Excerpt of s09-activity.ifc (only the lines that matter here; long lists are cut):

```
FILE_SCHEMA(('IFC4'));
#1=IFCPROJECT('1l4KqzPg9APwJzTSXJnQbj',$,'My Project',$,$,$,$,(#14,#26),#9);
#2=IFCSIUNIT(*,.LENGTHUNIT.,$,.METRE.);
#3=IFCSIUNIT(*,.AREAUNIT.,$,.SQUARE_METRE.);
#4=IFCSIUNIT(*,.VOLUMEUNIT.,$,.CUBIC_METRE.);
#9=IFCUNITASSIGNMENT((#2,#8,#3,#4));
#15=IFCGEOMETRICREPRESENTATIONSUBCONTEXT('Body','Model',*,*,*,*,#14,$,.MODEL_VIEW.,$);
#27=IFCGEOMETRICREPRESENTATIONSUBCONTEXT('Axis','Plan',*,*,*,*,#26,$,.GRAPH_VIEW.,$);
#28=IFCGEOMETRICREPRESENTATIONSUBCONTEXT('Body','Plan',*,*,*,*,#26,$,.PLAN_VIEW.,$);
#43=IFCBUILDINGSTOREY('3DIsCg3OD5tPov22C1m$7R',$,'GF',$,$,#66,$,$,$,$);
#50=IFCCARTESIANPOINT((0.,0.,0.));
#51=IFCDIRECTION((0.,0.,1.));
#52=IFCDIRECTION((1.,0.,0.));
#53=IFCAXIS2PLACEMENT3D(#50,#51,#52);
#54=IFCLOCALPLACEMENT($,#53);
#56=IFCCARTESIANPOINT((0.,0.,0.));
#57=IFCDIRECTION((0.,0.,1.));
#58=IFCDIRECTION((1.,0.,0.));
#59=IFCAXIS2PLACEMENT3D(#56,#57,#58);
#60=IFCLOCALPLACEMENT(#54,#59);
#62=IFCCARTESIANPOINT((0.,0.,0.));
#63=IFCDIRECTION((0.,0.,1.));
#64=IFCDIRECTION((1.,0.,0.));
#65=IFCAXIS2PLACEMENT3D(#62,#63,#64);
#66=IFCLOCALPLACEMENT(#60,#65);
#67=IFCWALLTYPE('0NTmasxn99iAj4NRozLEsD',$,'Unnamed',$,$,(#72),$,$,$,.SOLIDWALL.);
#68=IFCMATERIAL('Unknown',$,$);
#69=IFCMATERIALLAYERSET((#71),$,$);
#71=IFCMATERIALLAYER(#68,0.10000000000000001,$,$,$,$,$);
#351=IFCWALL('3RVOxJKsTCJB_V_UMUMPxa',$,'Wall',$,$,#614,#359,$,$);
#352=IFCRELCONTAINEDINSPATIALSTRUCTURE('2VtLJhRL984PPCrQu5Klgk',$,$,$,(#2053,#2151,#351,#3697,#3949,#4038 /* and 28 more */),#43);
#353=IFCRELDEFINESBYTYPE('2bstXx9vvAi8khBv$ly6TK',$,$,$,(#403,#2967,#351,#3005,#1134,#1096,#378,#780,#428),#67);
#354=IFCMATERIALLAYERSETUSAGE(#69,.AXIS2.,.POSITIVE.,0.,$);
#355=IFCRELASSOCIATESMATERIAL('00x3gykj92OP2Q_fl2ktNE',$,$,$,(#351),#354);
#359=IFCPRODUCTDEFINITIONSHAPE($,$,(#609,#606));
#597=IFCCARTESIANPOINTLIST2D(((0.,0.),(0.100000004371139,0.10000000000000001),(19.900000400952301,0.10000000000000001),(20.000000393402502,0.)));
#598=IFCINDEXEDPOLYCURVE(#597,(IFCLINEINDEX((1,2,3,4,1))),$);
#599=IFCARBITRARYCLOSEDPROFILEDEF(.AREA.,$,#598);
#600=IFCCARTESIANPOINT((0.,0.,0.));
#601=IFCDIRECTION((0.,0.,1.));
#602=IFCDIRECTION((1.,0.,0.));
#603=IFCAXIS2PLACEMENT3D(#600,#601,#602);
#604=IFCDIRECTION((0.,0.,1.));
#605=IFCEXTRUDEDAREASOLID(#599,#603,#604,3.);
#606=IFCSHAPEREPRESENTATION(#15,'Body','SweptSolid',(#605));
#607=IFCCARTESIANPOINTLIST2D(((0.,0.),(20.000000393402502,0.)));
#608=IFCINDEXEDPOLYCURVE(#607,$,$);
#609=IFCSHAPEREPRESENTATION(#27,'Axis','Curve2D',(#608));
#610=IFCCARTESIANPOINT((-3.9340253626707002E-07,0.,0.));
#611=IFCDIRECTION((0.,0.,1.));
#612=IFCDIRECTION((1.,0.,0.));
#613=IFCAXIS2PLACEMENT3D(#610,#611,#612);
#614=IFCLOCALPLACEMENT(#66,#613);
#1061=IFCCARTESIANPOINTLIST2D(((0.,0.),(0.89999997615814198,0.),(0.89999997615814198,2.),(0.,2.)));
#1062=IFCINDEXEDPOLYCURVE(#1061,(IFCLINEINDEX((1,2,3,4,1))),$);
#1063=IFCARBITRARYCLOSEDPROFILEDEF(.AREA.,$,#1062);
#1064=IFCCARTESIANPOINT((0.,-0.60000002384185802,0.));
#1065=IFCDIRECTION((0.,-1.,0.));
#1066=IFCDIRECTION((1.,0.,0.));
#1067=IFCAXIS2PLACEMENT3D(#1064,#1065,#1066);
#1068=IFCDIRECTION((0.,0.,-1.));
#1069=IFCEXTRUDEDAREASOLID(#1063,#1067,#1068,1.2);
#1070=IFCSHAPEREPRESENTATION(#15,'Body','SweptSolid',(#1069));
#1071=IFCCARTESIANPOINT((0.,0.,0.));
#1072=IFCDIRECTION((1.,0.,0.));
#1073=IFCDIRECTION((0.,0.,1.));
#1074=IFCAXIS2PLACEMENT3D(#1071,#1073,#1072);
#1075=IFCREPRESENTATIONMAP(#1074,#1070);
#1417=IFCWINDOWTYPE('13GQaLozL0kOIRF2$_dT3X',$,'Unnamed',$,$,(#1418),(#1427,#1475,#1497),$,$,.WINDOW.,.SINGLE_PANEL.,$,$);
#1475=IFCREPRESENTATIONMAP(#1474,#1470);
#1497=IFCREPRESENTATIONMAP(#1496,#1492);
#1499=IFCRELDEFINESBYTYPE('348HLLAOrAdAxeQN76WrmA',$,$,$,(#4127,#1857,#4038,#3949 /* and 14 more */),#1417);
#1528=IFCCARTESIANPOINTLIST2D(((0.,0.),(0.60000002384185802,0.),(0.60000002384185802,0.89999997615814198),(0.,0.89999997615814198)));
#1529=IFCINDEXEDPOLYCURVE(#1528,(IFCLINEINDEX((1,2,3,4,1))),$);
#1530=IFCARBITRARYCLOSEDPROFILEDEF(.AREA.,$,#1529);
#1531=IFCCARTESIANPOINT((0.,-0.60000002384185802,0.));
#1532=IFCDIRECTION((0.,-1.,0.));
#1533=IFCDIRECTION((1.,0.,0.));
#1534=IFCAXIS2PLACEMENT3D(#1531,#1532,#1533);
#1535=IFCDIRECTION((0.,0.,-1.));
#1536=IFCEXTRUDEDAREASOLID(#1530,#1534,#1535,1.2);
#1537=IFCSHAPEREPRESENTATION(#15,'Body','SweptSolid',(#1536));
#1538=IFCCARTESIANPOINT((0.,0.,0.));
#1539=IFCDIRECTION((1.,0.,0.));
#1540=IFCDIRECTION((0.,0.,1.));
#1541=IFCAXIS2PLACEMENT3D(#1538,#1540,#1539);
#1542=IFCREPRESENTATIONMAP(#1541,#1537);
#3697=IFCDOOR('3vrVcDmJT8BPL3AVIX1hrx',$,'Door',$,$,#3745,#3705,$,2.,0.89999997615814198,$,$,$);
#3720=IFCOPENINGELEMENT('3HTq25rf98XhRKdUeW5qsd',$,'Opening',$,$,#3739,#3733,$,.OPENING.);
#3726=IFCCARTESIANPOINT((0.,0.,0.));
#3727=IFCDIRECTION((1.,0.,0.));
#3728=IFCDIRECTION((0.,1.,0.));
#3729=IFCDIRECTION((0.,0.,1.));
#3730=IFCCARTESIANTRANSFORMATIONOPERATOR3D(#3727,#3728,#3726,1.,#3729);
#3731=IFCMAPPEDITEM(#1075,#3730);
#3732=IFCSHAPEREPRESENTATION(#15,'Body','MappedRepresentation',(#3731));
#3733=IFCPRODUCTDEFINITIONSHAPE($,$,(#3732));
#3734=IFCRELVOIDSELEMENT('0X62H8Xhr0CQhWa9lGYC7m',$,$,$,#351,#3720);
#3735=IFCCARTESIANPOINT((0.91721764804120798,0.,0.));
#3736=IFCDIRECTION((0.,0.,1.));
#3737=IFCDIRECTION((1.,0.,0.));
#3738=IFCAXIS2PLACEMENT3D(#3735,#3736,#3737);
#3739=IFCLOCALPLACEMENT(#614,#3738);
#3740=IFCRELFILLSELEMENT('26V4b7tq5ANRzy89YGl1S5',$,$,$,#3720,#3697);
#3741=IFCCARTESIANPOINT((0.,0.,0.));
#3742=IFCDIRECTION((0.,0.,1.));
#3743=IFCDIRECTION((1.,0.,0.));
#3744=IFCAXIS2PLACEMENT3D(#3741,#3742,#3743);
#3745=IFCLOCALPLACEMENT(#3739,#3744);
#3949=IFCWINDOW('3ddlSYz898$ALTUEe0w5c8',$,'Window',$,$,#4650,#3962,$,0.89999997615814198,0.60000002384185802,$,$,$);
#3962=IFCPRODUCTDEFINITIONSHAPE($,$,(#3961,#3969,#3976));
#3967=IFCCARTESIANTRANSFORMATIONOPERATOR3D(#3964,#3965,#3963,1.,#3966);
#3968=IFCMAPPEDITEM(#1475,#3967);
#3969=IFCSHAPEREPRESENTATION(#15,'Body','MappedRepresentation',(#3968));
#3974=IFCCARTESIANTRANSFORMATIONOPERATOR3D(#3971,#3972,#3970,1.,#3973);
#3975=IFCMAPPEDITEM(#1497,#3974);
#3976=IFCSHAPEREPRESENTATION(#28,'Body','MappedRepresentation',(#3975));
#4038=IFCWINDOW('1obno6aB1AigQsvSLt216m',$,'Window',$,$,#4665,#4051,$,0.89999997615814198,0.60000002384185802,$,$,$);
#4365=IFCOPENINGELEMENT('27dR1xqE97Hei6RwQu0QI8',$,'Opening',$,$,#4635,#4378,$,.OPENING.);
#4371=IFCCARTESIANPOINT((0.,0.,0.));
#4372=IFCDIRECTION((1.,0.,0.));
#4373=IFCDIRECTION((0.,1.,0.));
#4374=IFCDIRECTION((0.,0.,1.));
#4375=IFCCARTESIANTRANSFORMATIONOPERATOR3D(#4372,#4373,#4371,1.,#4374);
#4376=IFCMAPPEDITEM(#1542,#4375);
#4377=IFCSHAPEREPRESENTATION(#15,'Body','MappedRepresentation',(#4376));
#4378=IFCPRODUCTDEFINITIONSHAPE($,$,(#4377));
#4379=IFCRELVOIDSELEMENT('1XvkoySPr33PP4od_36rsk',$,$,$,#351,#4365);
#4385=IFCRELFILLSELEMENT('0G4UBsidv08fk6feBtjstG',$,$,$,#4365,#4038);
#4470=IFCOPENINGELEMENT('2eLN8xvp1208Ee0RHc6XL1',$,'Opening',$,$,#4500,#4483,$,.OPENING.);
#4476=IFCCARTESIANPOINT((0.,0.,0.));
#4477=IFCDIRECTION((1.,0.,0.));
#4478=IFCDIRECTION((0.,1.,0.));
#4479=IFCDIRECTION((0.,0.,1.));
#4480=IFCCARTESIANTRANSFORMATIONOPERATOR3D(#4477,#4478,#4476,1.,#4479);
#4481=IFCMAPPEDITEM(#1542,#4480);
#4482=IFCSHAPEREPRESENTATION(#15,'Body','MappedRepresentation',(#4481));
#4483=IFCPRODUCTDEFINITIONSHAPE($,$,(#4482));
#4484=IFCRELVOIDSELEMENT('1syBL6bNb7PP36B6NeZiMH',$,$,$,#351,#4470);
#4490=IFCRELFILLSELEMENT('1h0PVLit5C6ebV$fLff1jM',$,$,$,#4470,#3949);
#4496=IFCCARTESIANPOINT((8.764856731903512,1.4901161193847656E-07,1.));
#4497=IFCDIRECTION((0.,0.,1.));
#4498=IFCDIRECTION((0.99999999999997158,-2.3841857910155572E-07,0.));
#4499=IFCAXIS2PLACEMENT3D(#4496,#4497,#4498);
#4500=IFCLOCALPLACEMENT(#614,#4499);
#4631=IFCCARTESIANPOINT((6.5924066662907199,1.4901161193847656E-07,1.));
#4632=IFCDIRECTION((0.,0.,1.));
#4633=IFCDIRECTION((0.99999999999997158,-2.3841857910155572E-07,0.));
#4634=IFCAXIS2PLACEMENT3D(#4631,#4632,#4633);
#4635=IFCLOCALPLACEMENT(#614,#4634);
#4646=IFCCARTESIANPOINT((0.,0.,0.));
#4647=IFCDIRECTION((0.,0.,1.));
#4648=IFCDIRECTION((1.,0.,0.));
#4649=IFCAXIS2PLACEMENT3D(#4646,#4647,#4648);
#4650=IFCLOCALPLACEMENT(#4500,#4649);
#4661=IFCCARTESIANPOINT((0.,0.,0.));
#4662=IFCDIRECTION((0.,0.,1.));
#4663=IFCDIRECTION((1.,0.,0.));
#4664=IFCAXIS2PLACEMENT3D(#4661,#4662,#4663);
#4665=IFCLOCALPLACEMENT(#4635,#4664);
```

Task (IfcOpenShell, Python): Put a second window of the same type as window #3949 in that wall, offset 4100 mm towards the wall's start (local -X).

```python
import ifcopenshell
import ifcopenshell.api.feature
import ifcopenshell.api.geometry
import ifcopenshell.api.root
import ifcopenshell.geom
import ifcopenshell.util.element
import ifcopenshell.util.placement
import ifcopenshell.util.shape

model = ifcopenshell.open("s09-activity.ifc")
settings = ifcopenshell.geom.settings()


def volume(element):
    """Net volume in cubic metres, openings subtracted."""
    shape = ifcopenshell.geom.create_shape(settings, element)
    return ifcopenshell.util.shape.get_volume(shape.geometry)


window = model.by_id(3949)
opening = window.FillsVoids[0].RelatingOpeningElement
wall = opening.VoidsElements[0].RelatingBuildingElement
before = volume(wall)
shift = ifcopenshell.util.placement.get_local_placement(wall.ObjectPlacement)[:3, 0] * -4.1

# copy_class copies the void relationship, type, container and properties, but no geometry.
new_opening = ifcopenshell.api.root.copy_class(model, product=opening)
new_opening.Representation = ifcopenshell.util.element.copy_deep(
    model, opening.Representation, exclude=["IfcGeometricRepresentationContext", "IfcRepresentationMap"]
)
new_window = ifcopenshell.api.root.copy_class(model, product=window)
new_window.Representation = ifcopenshell.util.element.copy_deep(
    model, window.Representation, exclude=["IfcGeometricRepresentationContext", "IfcRepresentationMap"]
)
ifcopenshell.api.feature.add_filling(model, opening=new_opening, element=new_window)

for old, new in ((opening, new_opening), (window, new_window)):
    matrix = ifcopenshell.util.placement.get_local_placement(old.ObjectPlacement)
    matrix[:3, 3] += shift
    ifcopenshell.api.geometry.edit_object_placement(model, product=new, matrix=matrix, is_si=False)

after = volume(wall)

print(f"wall volume {before:.3f} -> {after:.3f} m3")

model.write("s09-activity_v2.ifc")
```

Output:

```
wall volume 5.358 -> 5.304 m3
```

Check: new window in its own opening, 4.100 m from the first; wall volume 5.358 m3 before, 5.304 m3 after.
